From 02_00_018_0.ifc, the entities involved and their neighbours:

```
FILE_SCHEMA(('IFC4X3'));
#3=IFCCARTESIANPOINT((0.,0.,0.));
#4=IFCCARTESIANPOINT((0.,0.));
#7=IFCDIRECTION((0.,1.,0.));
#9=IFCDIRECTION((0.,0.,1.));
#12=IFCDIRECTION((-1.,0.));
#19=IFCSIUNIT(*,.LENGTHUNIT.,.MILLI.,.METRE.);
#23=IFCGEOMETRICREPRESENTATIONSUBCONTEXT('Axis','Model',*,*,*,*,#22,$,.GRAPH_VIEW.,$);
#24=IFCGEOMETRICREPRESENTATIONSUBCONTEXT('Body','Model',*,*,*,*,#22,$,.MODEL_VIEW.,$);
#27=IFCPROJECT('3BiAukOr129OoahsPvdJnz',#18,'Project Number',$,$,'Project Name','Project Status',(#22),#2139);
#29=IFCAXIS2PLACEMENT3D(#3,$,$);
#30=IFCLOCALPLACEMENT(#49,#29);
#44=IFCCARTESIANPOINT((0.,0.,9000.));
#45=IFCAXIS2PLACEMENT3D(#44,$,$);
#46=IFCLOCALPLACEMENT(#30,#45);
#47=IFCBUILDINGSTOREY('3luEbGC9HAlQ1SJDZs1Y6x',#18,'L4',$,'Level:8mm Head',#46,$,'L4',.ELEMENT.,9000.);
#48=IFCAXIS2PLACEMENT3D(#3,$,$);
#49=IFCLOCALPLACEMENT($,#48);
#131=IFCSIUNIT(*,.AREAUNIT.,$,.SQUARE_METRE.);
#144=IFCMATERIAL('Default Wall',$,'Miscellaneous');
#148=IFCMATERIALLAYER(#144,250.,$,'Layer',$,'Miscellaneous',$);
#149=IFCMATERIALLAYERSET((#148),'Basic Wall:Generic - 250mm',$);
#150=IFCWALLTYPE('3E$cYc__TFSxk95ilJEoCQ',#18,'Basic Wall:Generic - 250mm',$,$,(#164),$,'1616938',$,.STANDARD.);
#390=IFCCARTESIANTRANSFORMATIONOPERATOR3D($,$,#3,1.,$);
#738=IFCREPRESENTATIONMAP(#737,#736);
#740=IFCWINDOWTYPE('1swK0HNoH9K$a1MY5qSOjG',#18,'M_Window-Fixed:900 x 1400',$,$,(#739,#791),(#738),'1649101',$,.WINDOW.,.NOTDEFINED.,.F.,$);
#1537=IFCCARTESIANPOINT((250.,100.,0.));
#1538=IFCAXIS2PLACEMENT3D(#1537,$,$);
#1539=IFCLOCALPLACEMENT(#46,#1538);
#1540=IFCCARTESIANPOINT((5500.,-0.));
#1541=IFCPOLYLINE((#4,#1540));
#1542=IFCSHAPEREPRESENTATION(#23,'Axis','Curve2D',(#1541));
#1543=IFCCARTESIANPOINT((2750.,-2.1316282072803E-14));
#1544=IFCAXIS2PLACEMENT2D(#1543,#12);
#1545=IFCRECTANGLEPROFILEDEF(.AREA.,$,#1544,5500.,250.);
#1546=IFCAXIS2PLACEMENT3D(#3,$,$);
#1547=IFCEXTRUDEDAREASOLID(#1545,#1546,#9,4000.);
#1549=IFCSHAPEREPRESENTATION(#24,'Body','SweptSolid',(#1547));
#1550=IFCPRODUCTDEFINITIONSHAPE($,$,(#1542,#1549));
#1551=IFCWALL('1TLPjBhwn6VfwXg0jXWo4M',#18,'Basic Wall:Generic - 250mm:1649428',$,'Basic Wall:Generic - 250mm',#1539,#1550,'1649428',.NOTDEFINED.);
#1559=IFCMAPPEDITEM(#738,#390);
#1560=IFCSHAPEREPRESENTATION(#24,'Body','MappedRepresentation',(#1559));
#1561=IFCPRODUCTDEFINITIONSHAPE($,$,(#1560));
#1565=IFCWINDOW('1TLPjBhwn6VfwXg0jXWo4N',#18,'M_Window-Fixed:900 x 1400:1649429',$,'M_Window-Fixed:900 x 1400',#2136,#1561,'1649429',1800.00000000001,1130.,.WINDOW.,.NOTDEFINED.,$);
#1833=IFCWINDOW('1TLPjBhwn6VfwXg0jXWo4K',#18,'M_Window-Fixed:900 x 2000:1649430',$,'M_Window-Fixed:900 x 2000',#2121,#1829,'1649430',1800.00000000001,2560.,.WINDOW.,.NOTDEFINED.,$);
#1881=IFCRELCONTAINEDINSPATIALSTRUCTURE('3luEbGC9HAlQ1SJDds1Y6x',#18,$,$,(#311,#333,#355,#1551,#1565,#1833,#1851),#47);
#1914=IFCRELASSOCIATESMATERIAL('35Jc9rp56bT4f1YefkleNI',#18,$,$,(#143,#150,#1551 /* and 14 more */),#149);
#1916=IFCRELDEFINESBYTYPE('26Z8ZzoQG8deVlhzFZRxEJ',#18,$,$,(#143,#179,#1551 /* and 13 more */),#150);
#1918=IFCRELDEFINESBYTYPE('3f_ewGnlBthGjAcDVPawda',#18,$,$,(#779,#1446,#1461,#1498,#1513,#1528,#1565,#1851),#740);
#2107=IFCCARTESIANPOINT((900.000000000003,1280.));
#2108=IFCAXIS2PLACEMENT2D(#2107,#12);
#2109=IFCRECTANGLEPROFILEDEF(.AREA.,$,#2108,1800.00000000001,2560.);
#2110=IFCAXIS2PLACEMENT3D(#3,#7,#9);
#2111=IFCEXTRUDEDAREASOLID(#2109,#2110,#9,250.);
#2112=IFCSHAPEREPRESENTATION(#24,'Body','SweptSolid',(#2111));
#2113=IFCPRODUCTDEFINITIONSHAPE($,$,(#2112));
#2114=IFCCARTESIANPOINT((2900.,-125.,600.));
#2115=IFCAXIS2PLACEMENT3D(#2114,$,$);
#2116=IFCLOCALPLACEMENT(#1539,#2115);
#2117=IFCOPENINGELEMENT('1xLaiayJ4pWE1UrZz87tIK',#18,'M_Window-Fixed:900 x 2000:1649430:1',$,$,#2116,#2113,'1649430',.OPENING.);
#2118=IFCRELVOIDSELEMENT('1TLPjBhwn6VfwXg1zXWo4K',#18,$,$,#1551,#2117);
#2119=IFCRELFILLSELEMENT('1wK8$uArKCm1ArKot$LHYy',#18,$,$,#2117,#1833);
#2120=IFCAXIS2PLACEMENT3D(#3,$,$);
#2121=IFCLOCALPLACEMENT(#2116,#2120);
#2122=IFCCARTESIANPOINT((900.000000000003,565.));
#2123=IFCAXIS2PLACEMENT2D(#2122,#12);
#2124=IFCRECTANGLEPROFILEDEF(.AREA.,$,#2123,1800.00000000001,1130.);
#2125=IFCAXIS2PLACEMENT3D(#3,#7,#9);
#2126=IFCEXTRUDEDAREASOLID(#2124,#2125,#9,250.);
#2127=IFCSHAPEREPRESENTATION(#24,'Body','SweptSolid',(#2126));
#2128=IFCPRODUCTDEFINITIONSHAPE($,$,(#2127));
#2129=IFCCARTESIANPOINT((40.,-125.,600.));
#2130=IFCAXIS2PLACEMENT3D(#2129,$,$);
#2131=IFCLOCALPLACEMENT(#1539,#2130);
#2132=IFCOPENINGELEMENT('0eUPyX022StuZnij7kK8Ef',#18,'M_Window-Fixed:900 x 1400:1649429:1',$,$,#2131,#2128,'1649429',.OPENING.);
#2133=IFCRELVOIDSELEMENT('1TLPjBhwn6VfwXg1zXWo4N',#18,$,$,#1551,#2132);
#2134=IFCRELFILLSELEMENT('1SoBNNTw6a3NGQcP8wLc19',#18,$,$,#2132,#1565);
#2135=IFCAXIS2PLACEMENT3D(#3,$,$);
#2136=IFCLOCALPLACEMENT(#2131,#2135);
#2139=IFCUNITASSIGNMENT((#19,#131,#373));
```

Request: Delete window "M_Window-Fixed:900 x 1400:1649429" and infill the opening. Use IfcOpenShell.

```python
import ifcopenshell
import ifcopenshell.api.feature
import ifcopenshell.api.root
import ifcopenshell.geom
import ifcopenshell.util.shape

model = ifcopenshell.open("02_00_018_0.ifc")
settings = ifcopenshell.geom.settings()


def volume(element):
    """Net volume in cubic metres, openings subtracted."""
    shape = ifcopenshell.geom.create_shape(settings, element)
    return ifcopenshell.util.shape.get_volume(shape.geometry)


window = model.by_id(1565)
opening = window.FillsVoids[0].RelatingOpeningElement
wall = opening.VoidsElements[0].RelatingBuildingElement
before = volume(wall)

ifcopenshell.api.root.remove_product(model, product=window)
ifcopenshell.api.feature.remove_feature(model, feature=opening)

after = volume(wall)

print(f"wall volume {before:.3f} -> {after:.3f} m3")

model.write("02_00_018_0_updated.ifc")
```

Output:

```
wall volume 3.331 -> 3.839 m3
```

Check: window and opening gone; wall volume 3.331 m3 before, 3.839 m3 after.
